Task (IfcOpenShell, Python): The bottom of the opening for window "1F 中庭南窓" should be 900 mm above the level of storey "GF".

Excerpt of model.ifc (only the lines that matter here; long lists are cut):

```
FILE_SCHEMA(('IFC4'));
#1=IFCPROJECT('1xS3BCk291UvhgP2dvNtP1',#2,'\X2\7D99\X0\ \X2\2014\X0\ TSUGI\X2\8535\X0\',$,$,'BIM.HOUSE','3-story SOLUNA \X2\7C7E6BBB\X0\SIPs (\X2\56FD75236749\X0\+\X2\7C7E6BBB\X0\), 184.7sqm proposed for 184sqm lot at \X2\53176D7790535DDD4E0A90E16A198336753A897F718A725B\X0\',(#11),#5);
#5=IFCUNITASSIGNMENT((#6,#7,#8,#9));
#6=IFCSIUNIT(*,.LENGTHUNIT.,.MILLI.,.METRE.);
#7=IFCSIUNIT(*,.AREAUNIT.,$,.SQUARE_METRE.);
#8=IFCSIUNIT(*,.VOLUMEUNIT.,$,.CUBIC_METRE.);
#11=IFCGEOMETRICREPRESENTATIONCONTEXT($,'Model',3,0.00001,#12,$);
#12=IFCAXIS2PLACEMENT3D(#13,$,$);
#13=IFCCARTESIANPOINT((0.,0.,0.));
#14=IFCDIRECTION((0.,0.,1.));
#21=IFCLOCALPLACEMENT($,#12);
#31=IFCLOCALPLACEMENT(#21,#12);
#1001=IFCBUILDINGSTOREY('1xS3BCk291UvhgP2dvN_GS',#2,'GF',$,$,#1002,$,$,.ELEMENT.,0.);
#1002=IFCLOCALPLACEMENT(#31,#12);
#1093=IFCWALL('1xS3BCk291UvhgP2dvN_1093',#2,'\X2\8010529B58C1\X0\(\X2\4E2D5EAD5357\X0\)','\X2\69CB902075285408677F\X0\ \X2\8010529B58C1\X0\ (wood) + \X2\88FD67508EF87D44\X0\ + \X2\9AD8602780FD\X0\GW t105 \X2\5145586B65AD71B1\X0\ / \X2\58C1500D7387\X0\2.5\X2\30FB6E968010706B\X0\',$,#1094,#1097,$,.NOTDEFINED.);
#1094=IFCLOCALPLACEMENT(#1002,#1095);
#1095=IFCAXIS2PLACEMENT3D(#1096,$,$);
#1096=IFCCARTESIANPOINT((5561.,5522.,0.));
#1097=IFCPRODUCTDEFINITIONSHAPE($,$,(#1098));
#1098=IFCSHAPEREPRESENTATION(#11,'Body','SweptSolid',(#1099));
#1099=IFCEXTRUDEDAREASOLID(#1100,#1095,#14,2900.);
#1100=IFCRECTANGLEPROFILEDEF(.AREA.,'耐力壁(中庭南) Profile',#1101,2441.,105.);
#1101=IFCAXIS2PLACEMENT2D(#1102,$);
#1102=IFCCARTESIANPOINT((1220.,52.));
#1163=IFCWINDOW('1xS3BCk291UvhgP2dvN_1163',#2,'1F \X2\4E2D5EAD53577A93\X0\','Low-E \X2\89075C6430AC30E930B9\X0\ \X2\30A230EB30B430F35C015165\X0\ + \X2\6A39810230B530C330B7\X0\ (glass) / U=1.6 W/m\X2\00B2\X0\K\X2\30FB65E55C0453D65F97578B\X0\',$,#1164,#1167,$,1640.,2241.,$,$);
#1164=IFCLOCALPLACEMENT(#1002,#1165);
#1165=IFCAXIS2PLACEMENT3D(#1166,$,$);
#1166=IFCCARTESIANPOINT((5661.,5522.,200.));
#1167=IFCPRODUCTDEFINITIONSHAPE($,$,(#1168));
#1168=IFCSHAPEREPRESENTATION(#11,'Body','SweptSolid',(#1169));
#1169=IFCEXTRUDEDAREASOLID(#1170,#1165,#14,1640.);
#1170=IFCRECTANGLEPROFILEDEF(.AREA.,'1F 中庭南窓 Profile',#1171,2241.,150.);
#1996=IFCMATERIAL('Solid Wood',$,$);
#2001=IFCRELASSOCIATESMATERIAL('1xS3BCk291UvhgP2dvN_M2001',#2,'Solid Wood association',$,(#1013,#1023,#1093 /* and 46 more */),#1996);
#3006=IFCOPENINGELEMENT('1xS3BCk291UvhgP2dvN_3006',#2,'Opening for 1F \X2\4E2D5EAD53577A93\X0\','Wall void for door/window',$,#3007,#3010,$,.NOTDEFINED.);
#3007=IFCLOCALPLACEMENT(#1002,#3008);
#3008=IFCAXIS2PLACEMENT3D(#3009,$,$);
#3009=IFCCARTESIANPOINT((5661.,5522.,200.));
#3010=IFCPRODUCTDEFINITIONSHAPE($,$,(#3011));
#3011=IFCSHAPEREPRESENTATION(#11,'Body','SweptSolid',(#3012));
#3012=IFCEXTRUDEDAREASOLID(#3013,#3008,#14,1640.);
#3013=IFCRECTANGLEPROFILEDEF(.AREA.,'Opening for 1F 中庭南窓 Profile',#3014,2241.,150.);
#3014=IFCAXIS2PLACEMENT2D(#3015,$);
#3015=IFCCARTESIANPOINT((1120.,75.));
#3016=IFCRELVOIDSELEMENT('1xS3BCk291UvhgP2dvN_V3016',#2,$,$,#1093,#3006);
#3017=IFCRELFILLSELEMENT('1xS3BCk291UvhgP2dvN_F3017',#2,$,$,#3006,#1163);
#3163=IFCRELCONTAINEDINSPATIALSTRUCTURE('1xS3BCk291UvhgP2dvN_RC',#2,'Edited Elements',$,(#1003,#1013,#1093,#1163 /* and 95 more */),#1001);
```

```python
import numpy as np
import ifcopenshell
import ifcopenshell.api.geometry
import ifcopenshell.geom
import ifcopenshell.util.element
import ifcopenshell.util.placement
import ifcopenshell.util.shape
import ifcopenshell.util.unit

model = ifcopenshell.open("model.ifc")
unit_scale = ifcopenshell.util.unit.calculate_unit_scale(model)

window = model.by_guid("1xS3BCk291UvhgP2dvN_1163")
opening = window.FillsVoids[0].RelatingOpeningElement
storey = ifcopenshell.util.element.get_container(window, ifc_class="IfcBuildingStorey")
level = ifcopenshell.util.placement.get_local_placement(storey.ObjectPlacement)[2, 3]

# The opening's origin need not be at the sill, so measure its lowest point.
shape = ifcopenshell.geom.create_shape(ifcopenshell.geom.settings(), opening)
bottom = ifcopenshell.util.shape.get_shape_bottom_elevation(shape, shape.geometry) / unit_scale
dz = level + 0.9 / unit_scale - bottom

shift = np.array([0.0, 0.0, dz])
# The window is not placed relative to its opening, so move both.
for product in (opening, window):
    matrix = ifcopenshell.util.placement.get_local_placement(product.ObjectPlacement)
    matrix[:3, 3] += shift
    ifcopenshell.api.geometry.edit_object_placement(model, product=product, matrix=matrix, is_si=False)

print(f"moved by {dz * unit_scale:+.3f} m")

model.write("model_edited.ifc")
```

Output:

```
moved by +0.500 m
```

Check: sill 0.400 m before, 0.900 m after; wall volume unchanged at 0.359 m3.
